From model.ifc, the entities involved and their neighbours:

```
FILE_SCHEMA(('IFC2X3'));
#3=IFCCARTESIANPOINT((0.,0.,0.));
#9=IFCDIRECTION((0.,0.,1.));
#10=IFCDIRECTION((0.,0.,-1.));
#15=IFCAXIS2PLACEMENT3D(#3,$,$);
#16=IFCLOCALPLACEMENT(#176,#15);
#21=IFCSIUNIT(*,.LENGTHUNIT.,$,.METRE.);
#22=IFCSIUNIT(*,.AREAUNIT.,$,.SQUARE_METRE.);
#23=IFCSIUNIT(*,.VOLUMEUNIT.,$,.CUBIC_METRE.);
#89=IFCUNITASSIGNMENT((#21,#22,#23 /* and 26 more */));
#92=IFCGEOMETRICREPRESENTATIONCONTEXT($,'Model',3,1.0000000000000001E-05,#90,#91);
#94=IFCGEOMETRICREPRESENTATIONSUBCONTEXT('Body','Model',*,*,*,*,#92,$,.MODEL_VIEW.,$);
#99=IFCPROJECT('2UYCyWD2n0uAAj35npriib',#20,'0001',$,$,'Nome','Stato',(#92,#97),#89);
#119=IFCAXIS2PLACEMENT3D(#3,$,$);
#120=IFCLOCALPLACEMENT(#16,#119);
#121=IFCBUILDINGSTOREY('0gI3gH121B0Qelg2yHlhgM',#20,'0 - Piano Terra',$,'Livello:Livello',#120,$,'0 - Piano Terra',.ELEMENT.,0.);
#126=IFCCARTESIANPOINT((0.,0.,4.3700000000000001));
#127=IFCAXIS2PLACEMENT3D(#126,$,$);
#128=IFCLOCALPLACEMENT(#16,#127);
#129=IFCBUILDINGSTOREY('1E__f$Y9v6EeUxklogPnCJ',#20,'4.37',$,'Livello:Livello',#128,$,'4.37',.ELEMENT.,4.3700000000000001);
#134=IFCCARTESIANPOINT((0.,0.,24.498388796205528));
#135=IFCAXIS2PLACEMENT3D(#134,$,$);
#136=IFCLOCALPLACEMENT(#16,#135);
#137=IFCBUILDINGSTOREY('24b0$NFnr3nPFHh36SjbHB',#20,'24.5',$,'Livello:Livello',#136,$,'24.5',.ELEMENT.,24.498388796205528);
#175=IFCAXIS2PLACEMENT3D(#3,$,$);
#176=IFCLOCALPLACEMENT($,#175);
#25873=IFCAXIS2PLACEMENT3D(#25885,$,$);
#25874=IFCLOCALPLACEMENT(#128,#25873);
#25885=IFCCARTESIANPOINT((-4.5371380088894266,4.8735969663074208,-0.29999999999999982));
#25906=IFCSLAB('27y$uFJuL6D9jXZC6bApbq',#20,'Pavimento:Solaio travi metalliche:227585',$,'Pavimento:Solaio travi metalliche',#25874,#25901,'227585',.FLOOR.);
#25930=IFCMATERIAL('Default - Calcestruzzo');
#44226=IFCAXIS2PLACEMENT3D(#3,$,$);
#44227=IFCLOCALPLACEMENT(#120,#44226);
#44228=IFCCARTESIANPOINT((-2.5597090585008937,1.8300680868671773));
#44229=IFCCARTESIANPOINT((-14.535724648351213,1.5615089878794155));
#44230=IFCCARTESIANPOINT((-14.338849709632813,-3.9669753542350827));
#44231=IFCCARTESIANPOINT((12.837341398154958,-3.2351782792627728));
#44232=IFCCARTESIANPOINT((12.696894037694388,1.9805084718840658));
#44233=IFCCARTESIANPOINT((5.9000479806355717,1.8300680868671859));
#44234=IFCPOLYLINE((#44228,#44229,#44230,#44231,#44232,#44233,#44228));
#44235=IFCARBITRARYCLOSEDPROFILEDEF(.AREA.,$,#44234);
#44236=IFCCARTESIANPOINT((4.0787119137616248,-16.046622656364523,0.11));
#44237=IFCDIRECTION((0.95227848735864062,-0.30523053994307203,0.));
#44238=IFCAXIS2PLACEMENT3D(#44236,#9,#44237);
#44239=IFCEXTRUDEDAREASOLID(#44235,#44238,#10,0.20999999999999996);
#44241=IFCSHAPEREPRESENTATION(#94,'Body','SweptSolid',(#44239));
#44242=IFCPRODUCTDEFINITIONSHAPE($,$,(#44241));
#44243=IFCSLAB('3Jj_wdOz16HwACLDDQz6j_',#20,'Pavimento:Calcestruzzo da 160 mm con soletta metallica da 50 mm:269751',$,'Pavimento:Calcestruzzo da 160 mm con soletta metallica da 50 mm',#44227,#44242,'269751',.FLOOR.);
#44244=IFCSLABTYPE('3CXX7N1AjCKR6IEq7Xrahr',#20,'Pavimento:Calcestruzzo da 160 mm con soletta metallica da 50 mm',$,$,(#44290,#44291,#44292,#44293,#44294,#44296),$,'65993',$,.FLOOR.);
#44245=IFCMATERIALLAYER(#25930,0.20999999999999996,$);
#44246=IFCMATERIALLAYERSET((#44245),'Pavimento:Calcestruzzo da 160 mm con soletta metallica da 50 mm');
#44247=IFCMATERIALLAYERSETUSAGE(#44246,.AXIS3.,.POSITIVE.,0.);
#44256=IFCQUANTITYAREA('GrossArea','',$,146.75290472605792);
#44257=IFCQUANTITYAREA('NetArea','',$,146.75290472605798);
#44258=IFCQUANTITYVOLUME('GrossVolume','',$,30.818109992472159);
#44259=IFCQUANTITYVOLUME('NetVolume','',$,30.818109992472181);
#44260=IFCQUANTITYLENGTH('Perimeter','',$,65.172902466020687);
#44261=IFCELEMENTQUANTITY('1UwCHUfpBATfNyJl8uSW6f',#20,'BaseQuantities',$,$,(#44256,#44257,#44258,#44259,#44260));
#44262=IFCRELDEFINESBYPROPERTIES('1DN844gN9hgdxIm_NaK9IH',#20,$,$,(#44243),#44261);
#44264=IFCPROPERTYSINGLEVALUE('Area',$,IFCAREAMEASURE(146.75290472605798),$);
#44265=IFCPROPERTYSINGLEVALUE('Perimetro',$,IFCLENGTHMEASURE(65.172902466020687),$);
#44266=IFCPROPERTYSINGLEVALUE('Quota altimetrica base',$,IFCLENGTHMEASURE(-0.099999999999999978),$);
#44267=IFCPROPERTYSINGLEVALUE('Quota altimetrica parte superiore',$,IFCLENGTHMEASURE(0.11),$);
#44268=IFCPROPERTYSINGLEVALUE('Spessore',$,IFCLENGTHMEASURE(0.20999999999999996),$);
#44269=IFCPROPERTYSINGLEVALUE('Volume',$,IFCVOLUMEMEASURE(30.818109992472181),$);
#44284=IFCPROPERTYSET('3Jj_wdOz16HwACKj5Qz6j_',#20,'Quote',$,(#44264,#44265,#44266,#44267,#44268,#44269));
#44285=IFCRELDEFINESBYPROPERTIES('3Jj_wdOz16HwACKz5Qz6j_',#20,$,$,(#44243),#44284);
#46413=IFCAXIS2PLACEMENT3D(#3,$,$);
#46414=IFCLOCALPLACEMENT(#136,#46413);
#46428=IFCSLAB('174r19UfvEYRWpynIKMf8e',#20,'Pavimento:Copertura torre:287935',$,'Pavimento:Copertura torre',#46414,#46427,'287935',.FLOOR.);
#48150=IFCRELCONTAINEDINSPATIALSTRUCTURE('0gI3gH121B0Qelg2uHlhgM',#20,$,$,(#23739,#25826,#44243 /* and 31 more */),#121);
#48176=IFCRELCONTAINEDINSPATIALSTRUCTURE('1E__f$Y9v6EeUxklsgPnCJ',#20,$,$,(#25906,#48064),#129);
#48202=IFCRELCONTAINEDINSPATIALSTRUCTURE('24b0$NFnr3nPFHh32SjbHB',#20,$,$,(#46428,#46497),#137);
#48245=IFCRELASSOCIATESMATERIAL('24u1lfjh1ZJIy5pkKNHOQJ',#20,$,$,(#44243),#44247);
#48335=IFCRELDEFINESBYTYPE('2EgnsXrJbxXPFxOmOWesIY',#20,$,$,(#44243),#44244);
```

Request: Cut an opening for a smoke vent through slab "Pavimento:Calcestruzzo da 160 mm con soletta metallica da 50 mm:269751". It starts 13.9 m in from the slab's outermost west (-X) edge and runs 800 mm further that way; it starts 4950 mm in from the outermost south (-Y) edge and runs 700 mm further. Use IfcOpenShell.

```python
import numpy as np
import ifcopenshell
import ifcopenshell.api.feature
import ifcopenshell.api.geometry
import ifcopenshell.api.pset
import ifcopenshell.api.root
import ifcopenshell.geom
import ifcopenshell.util.element
import ifcopenshell.util.placement
import ifcopenshell.util.representation
import ifcopenshell.util.shape
import ifcopenshell.util.unit

model = ifcopenshell.open("model.ifc")
unit_scale = ifcopenshell.util.unit.calculate_unit_scale(model)
area_scale = ifcopenshell.util.unit.calculate_unit_scale(model, "AREAUNIT")
volume_scale = ifcopenshell.util.unit.calculate_unit_scale(model, "VOLUMEUNIT")
settings = ifcopenshell.geom.settings()


def volume(element):
    """Net volume in cubic metres, openings subtracted."""
    shape = ifcopenshell.geom.create_shape(settings, element)
    return ifcopenshell.util.shape.get_volume(shape.geometry)


slab = model.by_id(44243)
before = volume(slab)

# Extent in the slab's own axes, in metres. The edges named are its -X and -Y sides.
slab_shape = ifcopenshell.geom.create_shape(settings, slab)
vertices = ifcopenshell.util.shape.get_vertices(slab_shape.geometry)
x_min, y_min, bottom = vertices.min(axis=0)
top = vertices[:, 2].max()

opening = ifcopenshell.api.root.create_entity(model, ifc_class="IfcOpeningElement", name="Smoke vent opening")
context = ifcopenshell.util.representation.get_context(model, "Model", "Body", "MODEL_VIEW")
width, depth = 0.8, 0.7
outline = [(0.0, 0.0), (width, 0.0), (width, depth), (0.0, depth), (0.0, 0.0)]
# Overshoot both faces by 50 mm so the cut is clean.
shape = ifcopenshell.api.geometry.add_slab_representation(
    model, context=context, depth=top - bottom + 0.1, polyline=outline
)
ifcopenshell.api.geometry.assign_representation(model, product=opening, representation=shape)

matrix = ifcopenshell.util.placement.get_local_placement(slab.ObjectPlacement)
matrix[:, 3] = matrix @ np.append(np.array([x_min + 13.9, y_min + 4.95, bottom - 0.05]) / unit_scale, 1.0)
ifcopenshell.api.geometry.edit_object_placement(model, product=opening, matrix=matrix, is_si=False)
ifcopenshell.api.feature.add_feature(model, feature=opening, element=slab)

after = volume(slab)

# Update the slab's stored quantities.
qto = model.by_id(ifcopenshell.util.element.get_pset(slab, "BaseQuantities", should_inherit=False)["id"])
ifcopenshell.api.pset.edit_qto(model, qto=qto, properties={
    "NetArea": after / (top - bottom) / area_scale,
    "NetVolume": after / volume_scale,
})
pset = model.by_id(ifcopenshell.util.element.get_pset(slab, "Quote", should_inherit=False)["id"])
ifcopenshell.api.pset.edit_pset(model, pset=pset, properties={
    "Area": model.create_entity("IfcAreaMeasure", after / (top - bottom) / area_scale),
    "Volume": model.create_entity("IfcVolumeMeasure", after / volume_scale),
})

print(f"slab volume {before:.3f} -> {after:.3f} m3")

model.write("model-out.ifc")
```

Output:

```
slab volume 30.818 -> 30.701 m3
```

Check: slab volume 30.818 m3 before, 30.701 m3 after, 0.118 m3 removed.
